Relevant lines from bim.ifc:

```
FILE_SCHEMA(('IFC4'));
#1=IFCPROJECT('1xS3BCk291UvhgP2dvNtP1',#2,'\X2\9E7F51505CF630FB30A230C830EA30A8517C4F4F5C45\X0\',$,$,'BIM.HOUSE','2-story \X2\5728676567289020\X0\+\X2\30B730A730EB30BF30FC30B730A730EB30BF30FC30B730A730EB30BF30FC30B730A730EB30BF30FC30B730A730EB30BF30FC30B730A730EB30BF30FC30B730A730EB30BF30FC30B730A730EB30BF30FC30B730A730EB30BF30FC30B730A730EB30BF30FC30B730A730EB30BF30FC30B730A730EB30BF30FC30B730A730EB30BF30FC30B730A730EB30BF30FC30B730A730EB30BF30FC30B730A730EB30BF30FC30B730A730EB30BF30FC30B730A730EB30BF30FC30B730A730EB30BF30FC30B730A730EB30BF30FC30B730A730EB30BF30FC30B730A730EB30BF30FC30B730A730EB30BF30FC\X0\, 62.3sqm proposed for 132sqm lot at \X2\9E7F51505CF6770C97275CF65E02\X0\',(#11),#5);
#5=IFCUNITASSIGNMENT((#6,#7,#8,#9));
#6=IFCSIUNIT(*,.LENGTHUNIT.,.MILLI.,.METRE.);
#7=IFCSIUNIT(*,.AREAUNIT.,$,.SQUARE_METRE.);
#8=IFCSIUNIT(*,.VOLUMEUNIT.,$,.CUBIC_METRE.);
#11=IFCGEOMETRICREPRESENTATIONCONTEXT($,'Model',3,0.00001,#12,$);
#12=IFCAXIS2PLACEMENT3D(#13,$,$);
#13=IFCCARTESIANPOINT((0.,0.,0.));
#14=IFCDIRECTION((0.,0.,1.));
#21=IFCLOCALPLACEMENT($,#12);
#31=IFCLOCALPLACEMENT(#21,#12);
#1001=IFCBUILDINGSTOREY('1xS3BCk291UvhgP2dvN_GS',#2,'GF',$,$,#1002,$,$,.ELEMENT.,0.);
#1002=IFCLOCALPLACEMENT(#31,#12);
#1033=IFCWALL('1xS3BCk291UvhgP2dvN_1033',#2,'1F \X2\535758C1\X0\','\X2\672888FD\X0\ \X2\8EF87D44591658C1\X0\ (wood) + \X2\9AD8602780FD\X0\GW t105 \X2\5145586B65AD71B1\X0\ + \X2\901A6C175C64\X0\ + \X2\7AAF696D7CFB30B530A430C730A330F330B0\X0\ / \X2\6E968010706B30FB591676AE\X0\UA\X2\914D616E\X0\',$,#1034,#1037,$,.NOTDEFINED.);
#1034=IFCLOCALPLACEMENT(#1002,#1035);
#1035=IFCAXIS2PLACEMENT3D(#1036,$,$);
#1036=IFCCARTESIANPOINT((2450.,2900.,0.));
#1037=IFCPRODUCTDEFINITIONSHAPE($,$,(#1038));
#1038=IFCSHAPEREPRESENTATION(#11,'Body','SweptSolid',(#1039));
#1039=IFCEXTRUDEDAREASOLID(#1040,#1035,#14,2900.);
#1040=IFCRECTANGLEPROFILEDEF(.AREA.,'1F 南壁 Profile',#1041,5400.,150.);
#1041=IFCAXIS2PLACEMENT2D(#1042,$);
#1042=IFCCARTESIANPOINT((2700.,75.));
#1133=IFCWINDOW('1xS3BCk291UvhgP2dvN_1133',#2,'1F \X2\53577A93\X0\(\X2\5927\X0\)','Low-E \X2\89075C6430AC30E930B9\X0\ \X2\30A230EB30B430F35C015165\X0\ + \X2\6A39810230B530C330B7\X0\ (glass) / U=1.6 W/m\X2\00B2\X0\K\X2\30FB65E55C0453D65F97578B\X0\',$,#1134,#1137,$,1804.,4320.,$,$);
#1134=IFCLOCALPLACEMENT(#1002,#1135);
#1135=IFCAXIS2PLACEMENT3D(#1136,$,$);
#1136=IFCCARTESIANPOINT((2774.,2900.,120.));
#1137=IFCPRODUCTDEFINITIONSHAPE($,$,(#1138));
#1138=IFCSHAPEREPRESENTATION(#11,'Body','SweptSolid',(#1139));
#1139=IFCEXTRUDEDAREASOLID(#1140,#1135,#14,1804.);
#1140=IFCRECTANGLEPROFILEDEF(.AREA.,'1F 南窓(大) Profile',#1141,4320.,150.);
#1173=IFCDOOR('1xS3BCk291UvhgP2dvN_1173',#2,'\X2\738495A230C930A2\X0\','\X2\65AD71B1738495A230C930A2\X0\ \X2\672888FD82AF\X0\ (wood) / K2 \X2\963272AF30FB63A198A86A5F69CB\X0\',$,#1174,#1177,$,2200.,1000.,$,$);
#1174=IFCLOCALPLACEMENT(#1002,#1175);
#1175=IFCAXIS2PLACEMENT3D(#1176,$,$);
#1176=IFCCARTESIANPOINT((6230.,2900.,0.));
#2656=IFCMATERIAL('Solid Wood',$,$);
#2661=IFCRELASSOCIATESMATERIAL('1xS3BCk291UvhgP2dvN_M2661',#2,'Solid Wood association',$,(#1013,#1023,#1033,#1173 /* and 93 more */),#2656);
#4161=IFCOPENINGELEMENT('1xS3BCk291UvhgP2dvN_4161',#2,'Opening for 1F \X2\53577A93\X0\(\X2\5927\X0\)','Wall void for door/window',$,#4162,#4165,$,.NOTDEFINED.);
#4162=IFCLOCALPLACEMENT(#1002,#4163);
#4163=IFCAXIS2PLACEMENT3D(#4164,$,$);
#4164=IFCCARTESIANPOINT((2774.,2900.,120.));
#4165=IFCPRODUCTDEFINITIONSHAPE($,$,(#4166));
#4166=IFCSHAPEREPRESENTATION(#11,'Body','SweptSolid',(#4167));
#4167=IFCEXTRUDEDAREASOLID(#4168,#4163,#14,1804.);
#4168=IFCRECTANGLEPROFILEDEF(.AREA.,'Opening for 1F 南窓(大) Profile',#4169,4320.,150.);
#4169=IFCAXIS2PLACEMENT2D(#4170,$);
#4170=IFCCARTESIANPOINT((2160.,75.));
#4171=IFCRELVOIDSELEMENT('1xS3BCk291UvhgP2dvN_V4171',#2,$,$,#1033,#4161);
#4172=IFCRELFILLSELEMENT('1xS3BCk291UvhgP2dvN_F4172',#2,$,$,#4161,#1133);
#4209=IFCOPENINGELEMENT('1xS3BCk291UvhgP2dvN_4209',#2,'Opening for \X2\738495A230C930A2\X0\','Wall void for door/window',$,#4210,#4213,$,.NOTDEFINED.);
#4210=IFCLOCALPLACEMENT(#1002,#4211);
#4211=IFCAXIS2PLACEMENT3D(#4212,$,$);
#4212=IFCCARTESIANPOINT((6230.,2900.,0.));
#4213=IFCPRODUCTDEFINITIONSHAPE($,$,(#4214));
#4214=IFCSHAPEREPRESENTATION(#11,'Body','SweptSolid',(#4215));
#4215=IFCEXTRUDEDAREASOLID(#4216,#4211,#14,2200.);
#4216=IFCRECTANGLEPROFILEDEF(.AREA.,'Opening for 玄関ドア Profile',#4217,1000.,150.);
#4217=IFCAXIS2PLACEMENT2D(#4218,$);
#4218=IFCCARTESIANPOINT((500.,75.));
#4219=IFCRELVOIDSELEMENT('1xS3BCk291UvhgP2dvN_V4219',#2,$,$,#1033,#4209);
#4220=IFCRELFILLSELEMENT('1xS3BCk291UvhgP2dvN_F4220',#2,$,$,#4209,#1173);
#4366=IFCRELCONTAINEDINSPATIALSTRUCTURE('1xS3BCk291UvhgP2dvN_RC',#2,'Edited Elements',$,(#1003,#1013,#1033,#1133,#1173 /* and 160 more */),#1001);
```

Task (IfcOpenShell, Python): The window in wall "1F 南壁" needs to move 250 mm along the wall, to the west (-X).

```python
import ifcopenshell
import ifcopenshell.api.geometry
import ifcopenshell.util.placement

model = ifcopenshell.open("bim.ifc")

window = model.by_guid("1xS3BCk291UvhgP2dvN_1133")
opening = window.FillsVoids[0].RelatingOpeningElement
wall = opening.VoidsElements[0].RelatingBuildingElement

wall_matrix = ifcopenshell.util.placement.get_local_placement(wall.ObjectPlacement)
shift = wall_matrix[:3, 0] * -250.0
before = ifcopenshell.util.placement.get_local_placement(window.ObjectPlacement)[:3, 3].copy()

# The window is not placed relative to its opening, so move both.
for product in (opening, window):
    matrix = ifcopenshell.util.placement.get_local_placement(product.ObjectPlacement)
    matrix[:3, 3] += shift
    ifcopenshell.api.geometry.edit_object_placement(model, product=product, matrix=matrix, is_si=False)

after = ifcopenshell.util.placement.get_local_placement(window.ObjectPlacement)[:3, 3]
print("window moved by", (after - before).round(3) + 0.0)

model.write("bim-out.ifc")
```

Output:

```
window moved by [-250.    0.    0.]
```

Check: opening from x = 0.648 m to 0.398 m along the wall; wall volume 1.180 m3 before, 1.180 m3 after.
